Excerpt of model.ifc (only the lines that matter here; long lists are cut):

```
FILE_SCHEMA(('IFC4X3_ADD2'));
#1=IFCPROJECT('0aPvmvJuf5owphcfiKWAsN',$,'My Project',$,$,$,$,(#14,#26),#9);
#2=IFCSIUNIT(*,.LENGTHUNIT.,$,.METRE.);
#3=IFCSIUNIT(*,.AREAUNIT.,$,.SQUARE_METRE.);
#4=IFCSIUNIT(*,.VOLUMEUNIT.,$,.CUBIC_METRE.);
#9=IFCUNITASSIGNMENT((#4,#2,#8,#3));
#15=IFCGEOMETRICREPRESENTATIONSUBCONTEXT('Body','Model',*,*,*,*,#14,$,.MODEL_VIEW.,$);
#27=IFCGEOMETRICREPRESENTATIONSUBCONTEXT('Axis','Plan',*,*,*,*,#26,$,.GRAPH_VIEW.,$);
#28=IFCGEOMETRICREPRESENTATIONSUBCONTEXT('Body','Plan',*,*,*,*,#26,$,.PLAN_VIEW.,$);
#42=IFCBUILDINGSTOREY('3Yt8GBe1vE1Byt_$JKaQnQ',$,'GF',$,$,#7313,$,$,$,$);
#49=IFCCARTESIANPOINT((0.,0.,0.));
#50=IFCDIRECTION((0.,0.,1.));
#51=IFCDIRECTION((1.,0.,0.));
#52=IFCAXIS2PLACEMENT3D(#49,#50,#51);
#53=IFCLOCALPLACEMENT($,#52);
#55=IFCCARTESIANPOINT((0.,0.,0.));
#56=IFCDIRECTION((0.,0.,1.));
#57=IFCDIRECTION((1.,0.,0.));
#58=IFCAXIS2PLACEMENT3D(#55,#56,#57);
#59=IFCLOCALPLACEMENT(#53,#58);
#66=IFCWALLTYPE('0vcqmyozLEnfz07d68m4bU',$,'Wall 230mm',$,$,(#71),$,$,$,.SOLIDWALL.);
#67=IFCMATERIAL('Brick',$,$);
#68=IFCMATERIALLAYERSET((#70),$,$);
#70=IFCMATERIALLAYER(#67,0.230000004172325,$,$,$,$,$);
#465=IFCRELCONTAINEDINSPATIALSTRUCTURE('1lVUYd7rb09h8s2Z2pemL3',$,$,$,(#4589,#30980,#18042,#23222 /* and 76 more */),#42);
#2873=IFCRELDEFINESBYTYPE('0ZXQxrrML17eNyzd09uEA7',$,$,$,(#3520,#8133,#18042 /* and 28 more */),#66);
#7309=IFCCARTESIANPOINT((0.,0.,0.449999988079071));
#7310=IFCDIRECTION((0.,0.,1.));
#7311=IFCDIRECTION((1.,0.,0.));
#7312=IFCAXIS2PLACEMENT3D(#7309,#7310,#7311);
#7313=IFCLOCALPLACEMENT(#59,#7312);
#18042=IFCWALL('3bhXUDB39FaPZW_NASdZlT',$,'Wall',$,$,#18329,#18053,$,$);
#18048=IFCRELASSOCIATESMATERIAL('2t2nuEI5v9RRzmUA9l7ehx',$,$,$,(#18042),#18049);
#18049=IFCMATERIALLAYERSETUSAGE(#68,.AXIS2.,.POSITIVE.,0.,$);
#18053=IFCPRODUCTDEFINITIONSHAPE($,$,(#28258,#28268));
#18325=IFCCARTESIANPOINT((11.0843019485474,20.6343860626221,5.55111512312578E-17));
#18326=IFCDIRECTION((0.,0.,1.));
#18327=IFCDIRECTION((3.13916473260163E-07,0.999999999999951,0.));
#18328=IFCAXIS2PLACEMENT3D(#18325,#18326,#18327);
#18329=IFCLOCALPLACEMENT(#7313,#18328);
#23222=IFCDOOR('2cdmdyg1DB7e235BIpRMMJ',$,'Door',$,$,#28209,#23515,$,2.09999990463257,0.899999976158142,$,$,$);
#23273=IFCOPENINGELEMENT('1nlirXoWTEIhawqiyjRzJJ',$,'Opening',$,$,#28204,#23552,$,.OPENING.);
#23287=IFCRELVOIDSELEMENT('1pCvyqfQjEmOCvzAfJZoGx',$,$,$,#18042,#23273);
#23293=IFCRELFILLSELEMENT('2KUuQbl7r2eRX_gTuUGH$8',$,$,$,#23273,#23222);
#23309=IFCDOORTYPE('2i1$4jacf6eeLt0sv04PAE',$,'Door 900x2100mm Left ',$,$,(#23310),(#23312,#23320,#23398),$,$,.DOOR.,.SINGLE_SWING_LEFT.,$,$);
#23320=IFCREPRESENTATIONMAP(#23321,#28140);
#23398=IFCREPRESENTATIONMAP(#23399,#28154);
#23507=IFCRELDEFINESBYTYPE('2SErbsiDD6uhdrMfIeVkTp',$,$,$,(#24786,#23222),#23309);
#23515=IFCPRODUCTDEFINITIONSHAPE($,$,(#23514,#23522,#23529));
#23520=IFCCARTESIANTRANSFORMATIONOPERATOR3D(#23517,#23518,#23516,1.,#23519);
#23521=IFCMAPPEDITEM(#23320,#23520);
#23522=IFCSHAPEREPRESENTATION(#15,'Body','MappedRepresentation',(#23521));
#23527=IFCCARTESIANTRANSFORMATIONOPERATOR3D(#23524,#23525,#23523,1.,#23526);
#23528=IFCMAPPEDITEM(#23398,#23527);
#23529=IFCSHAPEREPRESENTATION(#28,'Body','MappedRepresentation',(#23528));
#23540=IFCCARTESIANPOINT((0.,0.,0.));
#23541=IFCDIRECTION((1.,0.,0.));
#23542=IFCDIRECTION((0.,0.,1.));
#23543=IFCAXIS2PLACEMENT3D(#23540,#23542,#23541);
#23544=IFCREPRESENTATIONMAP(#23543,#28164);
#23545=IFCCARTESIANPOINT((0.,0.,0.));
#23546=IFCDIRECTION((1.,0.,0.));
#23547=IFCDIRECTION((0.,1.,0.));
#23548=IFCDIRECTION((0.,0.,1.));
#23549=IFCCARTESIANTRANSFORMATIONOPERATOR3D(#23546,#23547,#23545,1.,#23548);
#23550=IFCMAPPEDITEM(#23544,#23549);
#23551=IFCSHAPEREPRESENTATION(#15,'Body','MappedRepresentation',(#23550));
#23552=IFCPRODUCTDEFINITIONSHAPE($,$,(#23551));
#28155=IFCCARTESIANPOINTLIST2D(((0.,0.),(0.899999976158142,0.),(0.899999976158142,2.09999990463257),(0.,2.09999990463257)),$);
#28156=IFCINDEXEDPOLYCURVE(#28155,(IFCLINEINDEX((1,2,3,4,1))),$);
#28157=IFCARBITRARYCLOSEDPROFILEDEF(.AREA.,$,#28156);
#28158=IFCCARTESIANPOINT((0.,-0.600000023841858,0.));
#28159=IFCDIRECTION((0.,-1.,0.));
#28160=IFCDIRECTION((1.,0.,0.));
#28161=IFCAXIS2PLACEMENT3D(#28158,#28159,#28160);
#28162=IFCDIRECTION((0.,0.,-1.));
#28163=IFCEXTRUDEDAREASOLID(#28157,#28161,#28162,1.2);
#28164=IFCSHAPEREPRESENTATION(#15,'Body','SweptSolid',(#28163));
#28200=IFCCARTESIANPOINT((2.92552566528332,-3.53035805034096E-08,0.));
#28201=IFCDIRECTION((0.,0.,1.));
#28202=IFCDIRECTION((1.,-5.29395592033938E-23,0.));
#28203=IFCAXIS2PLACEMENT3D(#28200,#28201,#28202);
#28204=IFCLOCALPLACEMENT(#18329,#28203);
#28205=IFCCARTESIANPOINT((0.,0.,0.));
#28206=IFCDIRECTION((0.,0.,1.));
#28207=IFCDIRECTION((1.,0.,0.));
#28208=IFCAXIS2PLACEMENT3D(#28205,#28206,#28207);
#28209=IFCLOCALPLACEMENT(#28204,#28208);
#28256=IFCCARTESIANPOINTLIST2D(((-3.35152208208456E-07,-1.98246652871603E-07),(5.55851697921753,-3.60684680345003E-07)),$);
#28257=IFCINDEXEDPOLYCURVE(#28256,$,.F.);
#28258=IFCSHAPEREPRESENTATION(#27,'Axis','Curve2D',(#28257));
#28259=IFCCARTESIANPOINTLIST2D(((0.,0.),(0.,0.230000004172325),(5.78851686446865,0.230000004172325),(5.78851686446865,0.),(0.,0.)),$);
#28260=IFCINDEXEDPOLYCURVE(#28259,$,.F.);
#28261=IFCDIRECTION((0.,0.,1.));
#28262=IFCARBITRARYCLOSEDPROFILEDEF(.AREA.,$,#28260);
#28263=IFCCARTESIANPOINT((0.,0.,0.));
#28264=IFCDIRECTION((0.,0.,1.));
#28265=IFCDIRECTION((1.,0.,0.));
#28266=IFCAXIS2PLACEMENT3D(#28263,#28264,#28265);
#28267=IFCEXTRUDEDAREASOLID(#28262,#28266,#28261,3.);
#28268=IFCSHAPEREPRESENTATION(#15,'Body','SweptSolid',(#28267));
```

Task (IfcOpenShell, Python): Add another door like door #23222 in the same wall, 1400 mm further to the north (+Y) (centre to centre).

```python
import ifcopenshell
import ifcopenshell.api.feature
import ifcopenshell.api.geometry
import ifcopenshell.api.root
import ifcopenshell.geom
import ifcopenshell.util.element
import ifcopenshell.util.placement
import ifcopenshell.util.shape

model = ifcopenshell.open("model.ifc")
settings = ifcopenshell.geom.settings()


def volume(element):
    """Net volume in cubic metres, openings subtracted."""
    shape = ifcopenshell.geom.create_shape(settings, element)
    return ifcopenshell.util.shape.get_volume(shape.geometry)


door = model.by_id(23222)
opening = door.FillsVoids[0].RelatingOpeningElement
wall = opening.VoidsElements[0].RelatingBuildingElement
before = volume(wall)
shift = ifcopenshell.util.placement.get_local_placement(wall.ObjectPlacement)[:3, 0] * 1.4

# copy_class copies the void relationship, type, container and properties, but no geometry.
new_opening = ifcopenshell.api.root.copy_class(model, product=opening)
new_opening.Representation = ifcopenshell.util.element.copy_deep(
    model, opening.Representation, exclude=["IfcGeometricRepresentationContext", "IfcRepresentationMap"]
)
new_door = ifcopenshell.api.root.copy_class(model, product=door)
new_door.Representation = ifcopenshell.util.element.copy_deep(
    model, door.Representation, exclude=["IfcGeometricRepresentationContext", "IfcRepresentationMap"]
)
ifcopenshell.api.feature.add_filling(model, opening=new_opening, element=new_door)

for old, new in ((opening, new_opening), (door, new_door)):
    matrix = ifcopenshell.util.placement.get_local_placement(old.ObjectPlacement)
    matrix[:3, 3] += shift
    ifcopenshell.api.geometry.edit_object_placement(model, product=new, matrix=matrix, is_si=False)

after = volume(wall)

print(f"wall volume {before:.3f} -> {after:.3f} m3")

model.write("model_v2.ifc")
```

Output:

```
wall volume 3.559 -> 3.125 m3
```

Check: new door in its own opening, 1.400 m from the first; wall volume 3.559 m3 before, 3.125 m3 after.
